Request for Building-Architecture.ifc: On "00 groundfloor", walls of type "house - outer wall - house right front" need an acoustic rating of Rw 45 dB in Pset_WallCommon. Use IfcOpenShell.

First a look at what the model holds.

```python
import ifcopenshell
import ifcopenshell.util.element

model = ifcopenshell.open("Building-Architecture.ifc")
print(model.schema)
storey = next(s for s in model.by_type("IfcBuildingStorey") if s.Name == "00 groundfloor")
walls = [e for e in ifcopenshell.util.element.get_decomposition(storey) if e.is_a("IfcWall")]
seen = {}
for e in walls:
    element_type = ifcopenshell.util.element.get_type(e)
    key = (element_type.Name if element_type != e and element_type else None, ifcopenshell.util.element.get_pset(e, "Pset_WallCommon", "AcousticRating"))
    seen[key] = seen.get(key, 0) + 1
for (name, value), count in sorted(seen.items(), key=str):
    print(count, "x", name, "|", value)
```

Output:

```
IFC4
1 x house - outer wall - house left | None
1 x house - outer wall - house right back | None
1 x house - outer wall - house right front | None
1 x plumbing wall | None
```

```python
import ifcopenshell
import ifcopenshell.api.pset
import ifcopenshell.util.element

model = ifcopenshell.open("Building-Architecture.ifc")

storey = next(s for s in model.by_type("IfcBuildingStorey") if s.Name == "00 groundfloor")
walls = [e for e in ifcopenshell.util.element.get_decomposition(storey) if e.is_a("IfcWall")]

count = 0
for e in walls:
    element_type = ifcopenshell.util.element.get_type(e)
    if element_type in (None, e) or element_type.Name != "house - outer wall - house right front":
        continue
    # add_pset returns the element's existing set when there is one.
    pset = ifcopenshell.api.pset.add_pset(model, product=e, name="Pset_WallCommon")
    ifcopenshell.api.pset.edit_pset(model, pset=pset, properties={"AcousticRating": "Rw 45 dB"})
    count += 1

print(count, "walls updated")

model.write("Building-Architecture_updated.ifc")
```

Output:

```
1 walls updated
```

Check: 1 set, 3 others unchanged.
